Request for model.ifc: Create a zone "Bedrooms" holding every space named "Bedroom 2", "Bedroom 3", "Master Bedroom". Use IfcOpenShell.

First a look at what the model holds.

```python
import ifcopenshell

model = ifcopenshell.open("model.ifc")
print(model.schema)
seen = {}
for space in model.by_type("IfcSpace"):
    seen[space.LongName] = seen.get(space.LongName, 0) + 1
for name, count in sorted(seen.items(), key=str):
    print(count, "x", name)
print("zones:", [z.Name for z in model.by_type("IfcZone")][:20])
```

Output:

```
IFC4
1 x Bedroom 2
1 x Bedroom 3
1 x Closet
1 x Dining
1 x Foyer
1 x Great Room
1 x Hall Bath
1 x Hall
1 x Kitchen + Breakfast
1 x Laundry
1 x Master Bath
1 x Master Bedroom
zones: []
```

```python
import ifcopenshell
import ifcopenshell.api.group
import ifcopenshell.api.root

model = ifcopenshell.open("model.ifc")

names = {"Bedroom 2", "Bedroom 3", "Master Bedroom"}
spaces = [s for s in model.by_type("IfcSpace") if s.LongName in names]

zone = ifcopenshell.api.root.create_entity(model, ifc_class="IfcZone", name="Bedrooms")
ifcopenshell.api.group.assign_group(model, products=spaces, group=zone)
print(len(spaces), "spaces in", zone.Name)

model.write("model-out.ifc")
```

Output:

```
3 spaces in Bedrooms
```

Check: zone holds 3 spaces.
